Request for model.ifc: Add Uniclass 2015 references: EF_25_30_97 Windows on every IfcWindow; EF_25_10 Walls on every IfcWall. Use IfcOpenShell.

First a look at what the model holds.

```python
import ifcopenshell

model = ifcopenshell.open("model.ifc")
print(model.schema)
print("classifications:", [c.Name for c in model.by_type("IfcClassification")])
for ifc_class in ("IfcDoor", "IfcRoof", "IfcStair", "IfcWall", "IfcWindow"):
    print(ifc_class, len(model.by_type(ifc_class)))
```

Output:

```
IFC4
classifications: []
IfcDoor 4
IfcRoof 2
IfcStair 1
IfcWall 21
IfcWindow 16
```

```python
import ifcopenshell
import ifcopenshell.api.classification

model = ifcopenshell.open("model.ifc")

system = ifcopenshell.api.classification.add_classification(model, classification="Uniclass 2015")

codes = {
    "IfcWindow": ("EF_25_30_97", "Windows"),
    "IfcWall": ("EF_25_10", "Walls"),
}
for ifc_class, (code, name) in codes.items():
    products = model.by_type(ifc_class)
    ifcopenshell.api.classification.add_reference(
        model, products=products, classification=system, identification=code, name=name
    )
    print(code, len(products))

model.write("model-out.ifc")
```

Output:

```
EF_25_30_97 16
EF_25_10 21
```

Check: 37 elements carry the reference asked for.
